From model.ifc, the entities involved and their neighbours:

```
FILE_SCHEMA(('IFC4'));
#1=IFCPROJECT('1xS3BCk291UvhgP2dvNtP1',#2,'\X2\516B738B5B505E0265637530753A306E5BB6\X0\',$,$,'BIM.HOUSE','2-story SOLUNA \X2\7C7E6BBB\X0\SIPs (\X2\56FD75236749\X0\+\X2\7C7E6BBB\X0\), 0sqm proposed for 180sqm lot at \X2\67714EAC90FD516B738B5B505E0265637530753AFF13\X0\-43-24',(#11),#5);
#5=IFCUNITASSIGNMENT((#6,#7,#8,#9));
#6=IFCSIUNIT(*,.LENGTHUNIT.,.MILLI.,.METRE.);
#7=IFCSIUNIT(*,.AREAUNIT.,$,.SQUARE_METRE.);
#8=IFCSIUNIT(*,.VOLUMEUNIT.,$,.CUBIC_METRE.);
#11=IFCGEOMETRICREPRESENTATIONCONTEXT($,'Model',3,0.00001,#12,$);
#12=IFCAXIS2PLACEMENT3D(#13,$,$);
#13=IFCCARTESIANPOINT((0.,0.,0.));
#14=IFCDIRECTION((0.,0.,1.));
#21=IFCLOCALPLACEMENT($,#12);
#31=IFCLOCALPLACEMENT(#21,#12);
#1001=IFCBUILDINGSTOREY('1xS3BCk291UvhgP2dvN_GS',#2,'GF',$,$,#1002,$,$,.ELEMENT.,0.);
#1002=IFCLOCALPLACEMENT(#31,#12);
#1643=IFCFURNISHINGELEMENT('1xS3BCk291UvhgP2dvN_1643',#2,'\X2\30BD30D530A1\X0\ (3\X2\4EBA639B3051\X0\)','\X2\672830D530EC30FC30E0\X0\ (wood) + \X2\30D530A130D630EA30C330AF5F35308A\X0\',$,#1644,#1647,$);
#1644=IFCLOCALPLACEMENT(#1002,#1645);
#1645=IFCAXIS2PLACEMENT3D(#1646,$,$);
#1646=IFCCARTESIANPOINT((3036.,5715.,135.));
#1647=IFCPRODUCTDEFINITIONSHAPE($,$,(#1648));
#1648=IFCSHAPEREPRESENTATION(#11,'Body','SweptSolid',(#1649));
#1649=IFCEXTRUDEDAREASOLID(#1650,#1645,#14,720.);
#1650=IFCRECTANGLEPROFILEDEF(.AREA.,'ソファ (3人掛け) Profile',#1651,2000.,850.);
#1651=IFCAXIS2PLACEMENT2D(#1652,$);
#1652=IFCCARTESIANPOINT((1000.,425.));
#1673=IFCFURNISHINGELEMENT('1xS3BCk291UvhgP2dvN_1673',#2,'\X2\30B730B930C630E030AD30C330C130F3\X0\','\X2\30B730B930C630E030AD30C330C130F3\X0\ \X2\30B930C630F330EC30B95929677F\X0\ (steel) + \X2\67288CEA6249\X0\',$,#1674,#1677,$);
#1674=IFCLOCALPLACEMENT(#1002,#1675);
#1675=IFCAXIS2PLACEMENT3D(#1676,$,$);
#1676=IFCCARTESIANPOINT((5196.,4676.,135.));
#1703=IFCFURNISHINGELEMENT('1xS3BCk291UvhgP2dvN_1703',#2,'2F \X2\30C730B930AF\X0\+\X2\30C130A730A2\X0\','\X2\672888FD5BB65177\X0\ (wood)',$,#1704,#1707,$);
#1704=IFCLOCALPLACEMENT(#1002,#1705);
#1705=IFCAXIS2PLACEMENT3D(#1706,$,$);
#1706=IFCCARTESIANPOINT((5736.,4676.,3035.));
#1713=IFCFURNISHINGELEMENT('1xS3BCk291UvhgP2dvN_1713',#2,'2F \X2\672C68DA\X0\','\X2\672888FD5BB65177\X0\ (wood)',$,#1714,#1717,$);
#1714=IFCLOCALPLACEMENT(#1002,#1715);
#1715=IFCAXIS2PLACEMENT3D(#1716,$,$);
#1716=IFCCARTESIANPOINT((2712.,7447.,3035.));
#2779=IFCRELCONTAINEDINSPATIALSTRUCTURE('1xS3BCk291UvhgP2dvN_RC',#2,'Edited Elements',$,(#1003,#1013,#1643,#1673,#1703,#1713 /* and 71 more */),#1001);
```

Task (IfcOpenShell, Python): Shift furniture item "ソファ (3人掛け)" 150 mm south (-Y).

```python
import ifcopenshell
import ifcopenshell.api.geometry
import ifcopenshell.util.placement
import ifcopenshell.util.unit

model = ifcopenshell.open("model.ifc")
unit_scale = ifcopenshell.util.unit.calculate_unit_scale(model)

item = model.by_guid("1xS3BCk291UvhgP2dvN_1643")
matrix = ifcopenshell.util.placement.get_local_placement(item.ObjectPlacement)
matrix[1, 3] -= 0.15 / unit_scale
ifcopenshell.api.geometry.edit_object_placement(model, product=item, matrix=matrix, is_si=False)

print(ifcopenshell.util.placement.get_local_placement(item.ObjectPlacement).round(3) + 0.0)

model.write("model_edited.ifc")
```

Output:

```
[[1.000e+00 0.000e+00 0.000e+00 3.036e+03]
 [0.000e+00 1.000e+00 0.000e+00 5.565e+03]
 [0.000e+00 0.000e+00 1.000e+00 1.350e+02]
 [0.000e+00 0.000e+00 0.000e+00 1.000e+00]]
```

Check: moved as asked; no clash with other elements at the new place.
